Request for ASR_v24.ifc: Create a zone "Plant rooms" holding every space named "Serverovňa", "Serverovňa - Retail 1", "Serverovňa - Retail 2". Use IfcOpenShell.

First a look at what the model holds.

```python
import ifcopenshell

model = ifcopenshell.open("ASR_v24.ifc")
print(model.schema)
seen = {}
for space in model.by_type("IfcSpace"):
    seen[space.LongName] = seen.get(space.LongName, 0) + 1
for name, count in sorted(seen.items(), key=str):
    print(count, "x", name)
print("zones:", [z.Name for z in model.by_type("IfcZone")][:20])
```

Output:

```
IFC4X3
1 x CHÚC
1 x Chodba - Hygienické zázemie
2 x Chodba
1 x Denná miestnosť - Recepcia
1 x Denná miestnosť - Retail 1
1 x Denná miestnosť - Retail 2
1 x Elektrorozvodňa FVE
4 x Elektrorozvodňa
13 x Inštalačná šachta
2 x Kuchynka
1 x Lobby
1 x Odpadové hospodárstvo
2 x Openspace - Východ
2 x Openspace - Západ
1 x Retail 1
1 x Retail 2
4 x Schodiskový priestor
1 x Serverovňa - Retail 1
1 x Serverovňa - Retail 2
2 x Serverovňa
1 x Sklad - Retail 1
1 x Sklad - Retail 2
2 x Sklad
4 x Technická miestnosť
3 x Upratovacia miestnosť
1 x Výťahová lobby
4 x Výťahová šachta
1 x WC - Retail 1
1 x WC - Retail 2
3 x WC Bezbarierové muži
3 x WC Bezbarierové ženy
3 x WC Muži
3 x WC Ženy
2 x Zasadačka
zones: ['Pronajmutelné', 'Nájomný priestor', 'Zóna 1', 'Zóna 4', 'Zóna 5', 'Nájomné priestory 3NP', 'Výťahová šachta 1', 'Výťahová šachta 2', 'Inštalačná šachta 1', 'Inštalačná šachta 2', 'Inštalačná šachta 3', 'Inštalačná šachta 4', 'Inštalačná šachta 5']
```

```python
import ifcopenshell
import ifcopenshell.api.group
import ifcopenshell.api.root

model = ifcopenshell.open("ASR_v24.ifc")

names = {"Serverovňa", "Serverovňa - Retail 1", "Serverovňa - Retail 2"}
spaces = [s for s in model.by_type("IfcSpace") if s.LongName in names]

zone = ifcopenshell.api.root.create_entity(model, ifc_class="IfcZone", name="Plant rooms")
ifcopenshell.api.group.assign_group(model, products=spaces, group=zone)
print(len(spaces), "spaces in", zone.Name)

model.write("ASR_v24-out.ifc")
```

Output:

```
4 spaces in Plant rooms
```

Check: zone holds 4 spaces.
